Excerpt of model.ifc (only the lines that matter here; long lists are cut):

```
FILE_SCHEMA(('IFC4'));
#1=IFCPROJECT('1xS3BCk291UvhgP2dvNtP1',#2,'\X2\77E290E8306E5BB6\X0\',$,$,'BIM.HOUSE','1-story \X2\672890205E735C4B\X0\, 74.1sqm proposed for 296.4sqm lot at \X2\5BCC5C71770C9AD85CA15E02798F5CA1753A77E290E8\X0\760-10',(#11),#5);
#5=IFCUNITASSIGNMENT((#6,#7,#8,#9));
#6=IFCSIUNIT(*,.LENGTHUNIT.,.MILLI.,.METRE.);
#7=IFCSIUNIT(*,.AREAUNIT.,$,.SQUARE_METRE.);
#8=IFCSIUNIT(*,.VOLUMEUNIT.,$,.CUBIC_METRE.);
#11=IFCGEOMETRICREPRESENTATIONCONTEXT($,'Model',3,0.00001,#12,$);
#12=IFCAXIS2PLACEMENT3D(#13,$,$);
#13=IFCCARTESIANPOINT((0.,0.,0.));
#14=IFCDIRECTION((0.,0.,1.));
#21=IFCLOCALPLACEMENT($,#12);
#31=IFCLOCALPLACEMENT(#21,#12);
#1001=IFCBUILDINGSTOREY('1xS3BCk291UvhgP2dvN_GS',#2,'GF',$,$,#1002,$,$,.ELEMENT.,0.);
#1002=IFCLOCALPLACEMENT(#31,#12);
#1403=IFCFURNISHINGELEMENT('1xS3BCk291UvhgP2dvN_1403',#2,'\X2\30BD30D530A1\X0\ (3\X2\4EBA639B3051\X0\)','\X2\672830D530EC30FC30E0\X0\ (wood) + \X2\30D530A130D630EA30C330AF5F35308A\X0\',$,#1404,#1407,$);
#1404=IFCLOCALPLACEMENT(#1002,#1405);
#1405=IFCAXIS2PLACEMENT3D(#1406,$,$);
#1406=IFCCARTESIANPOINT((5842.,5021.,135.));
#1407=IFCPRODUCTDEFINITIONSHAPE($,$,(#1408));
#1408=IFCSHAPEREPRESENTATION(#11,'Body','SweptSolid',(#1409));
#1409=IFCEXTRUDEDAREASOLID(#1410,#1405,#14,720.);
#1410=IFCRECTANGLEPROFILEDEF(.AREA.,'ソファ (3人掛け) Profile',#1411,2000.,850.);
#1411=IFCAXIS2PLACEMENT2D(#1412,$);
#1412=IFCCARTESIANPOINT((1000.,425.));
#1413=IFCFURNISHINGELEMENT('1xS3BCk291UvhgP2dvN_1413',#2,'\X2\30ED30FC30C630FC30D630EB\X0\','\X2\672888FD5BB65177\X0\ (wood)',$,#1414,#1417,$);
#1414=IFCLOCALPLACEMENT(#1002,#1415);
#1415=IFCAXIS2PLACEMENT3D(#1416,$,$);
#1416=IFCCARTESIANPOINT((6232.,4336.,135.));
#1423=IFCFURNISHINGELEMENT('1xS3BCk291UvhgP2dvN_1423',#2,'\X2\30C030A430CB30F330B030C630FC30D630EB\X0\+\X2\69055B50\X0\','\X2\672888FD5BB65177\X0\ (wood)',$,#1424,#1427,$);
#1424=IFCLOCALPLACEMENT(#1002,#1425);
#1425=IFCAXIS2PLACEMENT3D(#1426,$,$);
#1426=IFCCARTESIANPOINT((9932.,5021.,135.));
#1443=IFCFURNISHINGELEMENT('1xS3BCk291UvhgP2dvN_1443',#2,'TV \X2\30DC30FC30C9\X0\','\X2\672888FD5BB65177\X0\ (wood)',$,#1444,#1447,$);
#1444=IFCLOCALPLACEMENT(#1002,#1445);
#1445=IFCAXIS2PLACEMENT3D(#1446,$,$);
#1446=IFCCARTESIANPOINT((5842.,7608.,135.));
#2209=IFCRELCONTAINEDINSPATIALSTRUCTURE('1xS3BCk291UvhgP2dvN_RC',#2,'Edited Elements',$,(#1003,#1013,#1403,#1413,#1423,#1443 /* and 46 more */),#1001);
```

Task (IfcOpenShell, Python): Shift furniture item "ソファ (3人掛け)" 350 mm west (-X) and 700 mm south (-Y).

```python
import ifcopenshell
import ifcopenshell.api.geometry
import ifcopenshell.util.placement
import ifcopenshell.util.unit

model = ifcopenshell.open("model.ifc")
unit_scale = ifcopenshell.util.unit.calculate_unit_scale(model)

item = model.by_guid("1xS3BCk291UvhgP2dvN_1403")
matrix = ifcopenshell.util.placement.get_local_placement(item.ObjectPlacement)
matrix[0, 3] -= 0.35 / unit_scale
matrix[1, 3] -= 0.7 / unit_scale
ifcopenshell.api.geometry.edit_object_placement(model, product=item, matrix=matrix, is_si=False)

print(ifcopenshell.util.placement.get_local_placement(item.ObjectPlacement).round(3) + 0.0)

model.write("model-out.ifc")
```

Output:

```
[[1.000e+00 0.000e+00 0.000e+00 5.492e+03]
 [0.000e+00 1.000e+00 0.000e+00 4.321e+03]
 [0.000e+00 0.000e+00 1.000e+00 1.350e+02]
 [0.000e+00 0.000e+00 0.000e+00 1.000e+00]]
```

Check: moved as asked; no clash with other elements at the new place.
